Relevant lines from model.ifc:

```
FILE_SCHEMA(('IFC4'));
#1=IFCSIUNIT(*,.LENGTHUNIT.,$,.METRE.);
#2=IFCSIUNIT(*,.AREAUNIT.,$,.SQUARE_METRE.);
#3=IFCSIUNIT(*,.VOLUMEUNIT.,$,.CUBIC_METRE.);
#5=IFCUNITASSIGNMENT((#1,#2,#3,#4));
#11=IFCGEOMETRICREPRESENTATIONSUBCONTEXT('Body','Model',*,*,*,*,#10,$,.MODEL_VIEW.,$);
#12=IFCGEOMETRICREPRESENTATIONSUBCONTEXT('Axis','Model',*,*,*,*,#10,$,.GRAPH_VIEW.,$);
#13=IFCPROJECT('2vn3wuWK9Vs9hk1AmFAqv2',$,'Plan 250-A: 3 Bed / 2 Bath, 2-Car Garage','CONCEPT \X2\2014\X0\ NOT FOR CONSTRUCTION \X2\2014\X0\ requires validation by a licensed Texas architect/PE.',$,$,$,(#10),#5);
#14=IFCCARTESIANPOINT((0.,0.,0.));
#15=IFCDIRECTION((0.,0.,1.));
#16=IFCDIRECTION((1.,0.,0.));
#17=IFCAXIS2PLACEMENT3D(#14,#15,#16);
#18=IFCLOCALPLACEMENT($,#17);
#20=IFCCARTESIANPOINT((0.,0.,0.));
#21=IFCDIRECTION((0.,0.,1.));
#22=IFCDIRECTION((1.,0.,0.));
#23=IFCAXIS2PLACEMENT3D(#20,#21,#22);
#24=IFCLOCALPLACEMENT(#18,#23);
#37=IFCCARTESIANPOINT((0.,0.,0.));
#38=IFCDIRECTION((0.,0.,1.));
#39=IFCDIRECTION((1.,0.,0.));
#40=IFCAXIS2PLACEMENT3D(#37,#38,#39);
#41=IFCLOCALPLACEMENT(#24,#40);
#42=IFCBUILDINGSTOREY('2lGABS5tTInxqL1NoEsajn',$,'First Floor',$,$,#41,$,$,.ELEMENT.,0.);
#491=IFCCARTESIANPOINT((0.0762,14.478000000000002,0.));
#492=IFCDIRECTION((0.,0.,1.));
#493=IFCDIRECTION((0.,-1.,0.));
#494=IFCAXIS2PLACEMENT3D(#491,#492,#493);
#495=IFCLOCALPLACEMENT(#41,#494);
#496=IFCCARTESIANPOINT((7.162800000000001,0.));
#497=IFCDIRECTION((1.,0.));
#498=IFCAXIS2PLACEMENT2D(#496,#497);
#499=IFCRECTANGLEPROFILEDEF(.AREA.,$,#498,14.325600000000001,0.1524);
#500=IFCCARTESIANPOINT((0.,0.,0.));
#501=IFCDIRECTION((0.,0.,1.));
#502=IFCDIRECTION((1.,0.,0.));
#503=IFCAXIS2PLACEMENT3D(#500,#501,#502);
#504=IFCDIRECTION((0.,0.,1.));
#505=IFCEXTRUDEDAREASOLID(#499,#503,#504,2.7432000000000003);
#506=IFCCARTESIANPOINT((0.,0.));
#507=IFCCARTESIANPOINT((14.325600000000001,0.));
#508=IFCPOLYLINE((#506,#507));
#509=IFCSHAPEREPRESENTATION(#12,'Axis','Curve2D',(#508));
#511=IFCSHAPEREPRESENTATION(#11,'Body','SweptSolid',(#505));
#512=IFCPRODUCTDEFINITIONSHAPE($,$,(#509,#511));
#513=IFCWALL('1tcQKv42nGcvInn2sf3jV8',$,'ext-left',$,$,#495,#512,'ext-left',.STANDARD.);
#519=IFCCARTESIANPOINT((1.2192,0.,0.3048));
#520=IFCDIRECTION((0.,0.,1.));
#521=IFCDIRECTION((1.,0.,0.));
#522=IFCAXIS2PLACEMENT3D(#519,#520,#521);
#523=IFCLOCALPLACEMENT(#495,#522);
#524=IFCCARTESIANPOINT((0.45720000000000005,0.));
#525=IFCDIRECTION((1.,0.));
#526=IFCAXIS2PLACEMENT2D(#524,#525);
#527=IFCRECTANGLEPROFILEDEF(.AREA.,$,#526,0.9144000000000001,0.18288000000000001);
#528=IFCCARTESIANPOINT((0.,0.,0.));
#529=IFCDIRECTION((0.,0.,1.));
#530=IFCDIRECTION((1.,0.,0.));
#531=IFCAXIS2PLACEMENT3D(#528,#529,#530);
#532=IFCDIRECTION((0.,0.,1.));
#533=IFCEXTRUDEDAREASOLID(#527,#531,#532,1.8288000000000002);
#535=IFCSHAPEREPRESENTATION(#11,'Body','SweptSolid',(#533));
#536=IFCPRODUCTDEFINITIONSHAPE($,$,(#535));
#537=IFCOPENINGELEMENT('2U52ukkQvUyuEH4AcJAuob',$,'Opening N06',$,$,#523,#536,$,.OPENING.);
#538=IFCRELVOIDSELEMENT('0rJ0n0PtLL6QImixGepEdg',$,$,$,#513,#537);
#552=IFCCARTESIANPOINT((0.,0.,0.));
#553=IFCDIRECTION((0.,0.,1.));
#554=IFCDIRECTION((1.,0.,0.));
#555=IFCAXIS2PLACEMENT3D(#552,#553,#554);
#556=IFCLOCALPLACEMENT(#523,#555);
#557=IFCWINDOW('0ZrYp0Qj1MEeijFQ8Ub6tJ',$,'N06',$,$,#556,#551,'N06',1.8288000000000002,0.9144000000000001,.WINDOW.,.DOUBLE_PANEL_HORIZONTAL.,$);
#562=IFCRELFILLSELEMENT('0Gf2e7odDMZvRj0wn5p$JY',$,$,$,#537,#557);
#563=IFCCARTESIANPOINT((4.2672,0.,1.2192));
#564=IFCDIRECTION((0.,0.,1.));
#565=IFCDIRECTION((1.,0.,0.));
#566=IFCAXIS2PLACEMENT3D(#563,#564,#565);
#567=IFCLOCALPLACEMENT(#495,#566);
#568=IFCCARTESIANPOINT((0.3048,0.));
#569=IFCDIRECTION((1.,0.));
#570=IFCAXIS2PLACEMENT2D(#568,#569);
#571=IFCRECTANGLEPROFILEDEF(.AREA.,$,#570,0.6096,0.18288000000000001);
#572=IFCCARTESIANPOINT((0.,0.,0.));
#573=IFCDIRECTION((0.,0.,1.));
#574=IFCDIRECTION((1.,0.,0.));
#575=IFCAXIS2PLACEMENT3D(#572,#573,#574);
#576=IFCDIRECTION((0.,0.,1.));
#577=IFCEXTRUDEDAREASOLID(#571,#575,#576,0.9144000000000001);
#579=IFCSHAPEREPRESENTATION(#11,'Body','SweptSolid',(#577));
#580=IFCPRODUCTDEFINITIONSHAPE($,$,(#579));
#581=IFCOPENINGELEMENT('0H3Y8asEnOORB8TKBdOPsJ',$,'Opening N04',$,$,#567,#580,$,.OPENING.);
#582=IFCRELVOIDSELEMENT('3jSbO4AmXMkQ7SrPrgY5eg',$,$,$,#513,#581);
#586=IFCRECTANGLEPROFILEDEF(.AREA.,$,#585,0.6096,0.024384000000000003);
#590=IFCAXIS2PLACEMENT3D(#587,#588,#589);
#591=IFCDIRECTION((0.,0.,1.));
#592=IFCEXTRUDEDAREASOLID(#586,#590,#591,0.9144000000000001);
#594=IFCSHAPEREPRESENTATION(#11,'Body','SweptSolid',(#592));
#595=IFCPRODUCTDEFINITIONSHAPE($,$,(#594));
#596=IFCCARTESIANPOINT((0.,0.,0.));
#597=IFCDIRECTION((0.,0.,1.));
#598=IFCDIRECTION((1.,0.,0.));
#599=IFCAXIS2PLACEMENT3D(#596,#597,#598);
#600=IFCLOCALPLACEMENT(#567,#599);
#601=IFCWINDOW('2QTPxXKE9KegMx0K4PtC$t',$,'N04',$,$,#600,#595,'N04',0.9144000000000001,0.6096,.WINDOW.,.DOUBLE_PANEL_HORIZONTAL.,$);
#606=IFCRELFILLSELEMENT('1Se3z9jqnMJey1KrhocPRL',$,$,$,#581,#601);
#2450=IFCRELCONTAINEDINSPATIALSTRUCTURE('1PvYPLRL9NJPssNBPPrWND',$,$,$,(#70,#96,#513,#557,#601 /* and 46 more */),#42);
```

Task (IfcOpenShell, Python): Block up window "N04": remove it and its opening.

```python
import ifcopenshell
import ifcopenshell.api.feature
import ifcopenshell.api.root
import ifcopenshell.geom
import ifcopenshell.util.shape

model = ifcopenshell.open("model.ifc")
settings = ifcopenshell.geom.settings()


def volume(element):
    """Net volume in cubic metres, openings subtracted."""
    shape = ifcopenshell.geom.create_shape(settings, element)
    return ifcopenshell.util.shape.get_volume(shape.geometry)


window = model.by_guid("2QTPxXKE9KegMx0K4PtC$t")
opening = window.FillsVoids[0].RelatingOpeningElement
wall = opening.VoidsElements[0].RelatingBuildingElement
before = volume(wall)

ifcopenshell.api.root.remove_product(model, product=window)
ifcopenshell.api.feature.remove_feature(model, feature=opening)

after = volume(wall)

print(f"wall volume {before:.3f} -> {after:.3f} m3")

model.write("model_rev.ifc")
```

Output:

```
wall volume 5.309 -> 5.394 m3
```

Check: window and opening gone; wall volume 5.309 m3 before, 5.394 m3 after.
